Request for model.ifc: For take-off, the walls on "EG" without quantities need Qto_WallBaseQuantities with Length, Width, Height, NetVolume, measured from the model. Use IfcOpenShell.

First a look at what the model holds.

```python
import ifcopenshell
import ifcopenshell.util.element
import ifcopenshell.util.unit

model = ifcopenshell.open("model.ifc")
print(model.schema)
for unit_type in ("LENGTHUNIT", "AREAUNIT", "VOLUMEUNIT"):
    print(unit_type, ifcopenshell.util.unit.calculate_unit_scale(model, unit_type))
storey = next(s for s in model.by_type("IfcBuildingStorey") if s.Name == "EG")
walls = [e for e in ifcopenshell.util.element.get_decomposition(storey) if e.is_a("IfcWall")]
for e in sorted(walls, key=lambda e: e.id()):
    print(e.id(), e.is_a(), e.Name, list(ifcopenshell.util.element.get_psets(e, qtos_only=True)), sep=" | ")
```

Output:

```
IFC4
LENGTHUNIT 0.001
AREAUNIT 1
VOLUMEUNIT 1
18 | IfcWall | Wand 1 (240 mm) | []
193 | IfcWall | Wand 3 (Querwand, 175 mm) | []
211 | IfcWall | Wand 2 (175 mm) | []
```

```python
import ifcopenshell
import ifcopenshell.api.pset
import ifcopenshell.geom
import ifcopenshell.util.element
import ifcopenshell.util.shape
import ifcopenshell.util.unit

model = ifcopenshell.open("model.ifc")
unit_scale = ifcopenshell.util.unit.calculate_unit_scale(model)
volume_scale = ifcopenshell.util.unit.calculate_unit_scale(model, "VOLUMEUNIT")
settings = ifcopenshell.geom.settings()

storey = next(s for s in model.by_type("IfcBuildingStorey") if s.Name == "EG")
walls = [e for e in ifcopenshell.util.element.get_decomposition(storey) if e.is_a("IfcWall")]

for e in sorted(walls, key=lambda e: e.id()):
    if ifcopenshell.util.element.get_psets(e, qtos_only=True, should_inherit=False):
        continue
    # Geometry comes back in metres, in the element's own axes.
    shape = ifcopenshell.geom.create_shape(settings, e)
    values = {
        "Length": ifcopenshell.util.shape.get_x(shape.geometry) / unit_scale,
        "Width": ifcopenshell.util.shape.get_y(shape.geometry) / unit_scale,
        "Height": ifcopenshell.util.shape.get_z(shape.geometry) / unit_scale,
        "NetVolume": ifcopenshell.util.shape.get_volume(shape.geometry) / volume_scale,
    }
    qto = ifcopenshell.api.pset.add_qto(model, product=e, name="Qto_WallBaseQuantities")
    ifcopenshell.api.pset.edit_qto(model, qto=qto, properties=values)
    print(e.id(), {k: round(v, 3) for k, v in values.items()})

model.write("model_rev.ifc")
```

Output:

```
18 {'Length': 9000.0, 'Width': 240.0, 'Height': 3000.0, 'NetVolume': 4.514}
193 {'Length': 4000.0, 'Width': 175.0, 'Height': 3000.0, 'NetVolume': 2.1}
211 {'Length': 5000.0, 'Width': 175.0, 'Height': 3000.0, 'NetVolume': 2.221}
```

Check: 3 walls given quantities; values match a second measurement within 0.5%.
